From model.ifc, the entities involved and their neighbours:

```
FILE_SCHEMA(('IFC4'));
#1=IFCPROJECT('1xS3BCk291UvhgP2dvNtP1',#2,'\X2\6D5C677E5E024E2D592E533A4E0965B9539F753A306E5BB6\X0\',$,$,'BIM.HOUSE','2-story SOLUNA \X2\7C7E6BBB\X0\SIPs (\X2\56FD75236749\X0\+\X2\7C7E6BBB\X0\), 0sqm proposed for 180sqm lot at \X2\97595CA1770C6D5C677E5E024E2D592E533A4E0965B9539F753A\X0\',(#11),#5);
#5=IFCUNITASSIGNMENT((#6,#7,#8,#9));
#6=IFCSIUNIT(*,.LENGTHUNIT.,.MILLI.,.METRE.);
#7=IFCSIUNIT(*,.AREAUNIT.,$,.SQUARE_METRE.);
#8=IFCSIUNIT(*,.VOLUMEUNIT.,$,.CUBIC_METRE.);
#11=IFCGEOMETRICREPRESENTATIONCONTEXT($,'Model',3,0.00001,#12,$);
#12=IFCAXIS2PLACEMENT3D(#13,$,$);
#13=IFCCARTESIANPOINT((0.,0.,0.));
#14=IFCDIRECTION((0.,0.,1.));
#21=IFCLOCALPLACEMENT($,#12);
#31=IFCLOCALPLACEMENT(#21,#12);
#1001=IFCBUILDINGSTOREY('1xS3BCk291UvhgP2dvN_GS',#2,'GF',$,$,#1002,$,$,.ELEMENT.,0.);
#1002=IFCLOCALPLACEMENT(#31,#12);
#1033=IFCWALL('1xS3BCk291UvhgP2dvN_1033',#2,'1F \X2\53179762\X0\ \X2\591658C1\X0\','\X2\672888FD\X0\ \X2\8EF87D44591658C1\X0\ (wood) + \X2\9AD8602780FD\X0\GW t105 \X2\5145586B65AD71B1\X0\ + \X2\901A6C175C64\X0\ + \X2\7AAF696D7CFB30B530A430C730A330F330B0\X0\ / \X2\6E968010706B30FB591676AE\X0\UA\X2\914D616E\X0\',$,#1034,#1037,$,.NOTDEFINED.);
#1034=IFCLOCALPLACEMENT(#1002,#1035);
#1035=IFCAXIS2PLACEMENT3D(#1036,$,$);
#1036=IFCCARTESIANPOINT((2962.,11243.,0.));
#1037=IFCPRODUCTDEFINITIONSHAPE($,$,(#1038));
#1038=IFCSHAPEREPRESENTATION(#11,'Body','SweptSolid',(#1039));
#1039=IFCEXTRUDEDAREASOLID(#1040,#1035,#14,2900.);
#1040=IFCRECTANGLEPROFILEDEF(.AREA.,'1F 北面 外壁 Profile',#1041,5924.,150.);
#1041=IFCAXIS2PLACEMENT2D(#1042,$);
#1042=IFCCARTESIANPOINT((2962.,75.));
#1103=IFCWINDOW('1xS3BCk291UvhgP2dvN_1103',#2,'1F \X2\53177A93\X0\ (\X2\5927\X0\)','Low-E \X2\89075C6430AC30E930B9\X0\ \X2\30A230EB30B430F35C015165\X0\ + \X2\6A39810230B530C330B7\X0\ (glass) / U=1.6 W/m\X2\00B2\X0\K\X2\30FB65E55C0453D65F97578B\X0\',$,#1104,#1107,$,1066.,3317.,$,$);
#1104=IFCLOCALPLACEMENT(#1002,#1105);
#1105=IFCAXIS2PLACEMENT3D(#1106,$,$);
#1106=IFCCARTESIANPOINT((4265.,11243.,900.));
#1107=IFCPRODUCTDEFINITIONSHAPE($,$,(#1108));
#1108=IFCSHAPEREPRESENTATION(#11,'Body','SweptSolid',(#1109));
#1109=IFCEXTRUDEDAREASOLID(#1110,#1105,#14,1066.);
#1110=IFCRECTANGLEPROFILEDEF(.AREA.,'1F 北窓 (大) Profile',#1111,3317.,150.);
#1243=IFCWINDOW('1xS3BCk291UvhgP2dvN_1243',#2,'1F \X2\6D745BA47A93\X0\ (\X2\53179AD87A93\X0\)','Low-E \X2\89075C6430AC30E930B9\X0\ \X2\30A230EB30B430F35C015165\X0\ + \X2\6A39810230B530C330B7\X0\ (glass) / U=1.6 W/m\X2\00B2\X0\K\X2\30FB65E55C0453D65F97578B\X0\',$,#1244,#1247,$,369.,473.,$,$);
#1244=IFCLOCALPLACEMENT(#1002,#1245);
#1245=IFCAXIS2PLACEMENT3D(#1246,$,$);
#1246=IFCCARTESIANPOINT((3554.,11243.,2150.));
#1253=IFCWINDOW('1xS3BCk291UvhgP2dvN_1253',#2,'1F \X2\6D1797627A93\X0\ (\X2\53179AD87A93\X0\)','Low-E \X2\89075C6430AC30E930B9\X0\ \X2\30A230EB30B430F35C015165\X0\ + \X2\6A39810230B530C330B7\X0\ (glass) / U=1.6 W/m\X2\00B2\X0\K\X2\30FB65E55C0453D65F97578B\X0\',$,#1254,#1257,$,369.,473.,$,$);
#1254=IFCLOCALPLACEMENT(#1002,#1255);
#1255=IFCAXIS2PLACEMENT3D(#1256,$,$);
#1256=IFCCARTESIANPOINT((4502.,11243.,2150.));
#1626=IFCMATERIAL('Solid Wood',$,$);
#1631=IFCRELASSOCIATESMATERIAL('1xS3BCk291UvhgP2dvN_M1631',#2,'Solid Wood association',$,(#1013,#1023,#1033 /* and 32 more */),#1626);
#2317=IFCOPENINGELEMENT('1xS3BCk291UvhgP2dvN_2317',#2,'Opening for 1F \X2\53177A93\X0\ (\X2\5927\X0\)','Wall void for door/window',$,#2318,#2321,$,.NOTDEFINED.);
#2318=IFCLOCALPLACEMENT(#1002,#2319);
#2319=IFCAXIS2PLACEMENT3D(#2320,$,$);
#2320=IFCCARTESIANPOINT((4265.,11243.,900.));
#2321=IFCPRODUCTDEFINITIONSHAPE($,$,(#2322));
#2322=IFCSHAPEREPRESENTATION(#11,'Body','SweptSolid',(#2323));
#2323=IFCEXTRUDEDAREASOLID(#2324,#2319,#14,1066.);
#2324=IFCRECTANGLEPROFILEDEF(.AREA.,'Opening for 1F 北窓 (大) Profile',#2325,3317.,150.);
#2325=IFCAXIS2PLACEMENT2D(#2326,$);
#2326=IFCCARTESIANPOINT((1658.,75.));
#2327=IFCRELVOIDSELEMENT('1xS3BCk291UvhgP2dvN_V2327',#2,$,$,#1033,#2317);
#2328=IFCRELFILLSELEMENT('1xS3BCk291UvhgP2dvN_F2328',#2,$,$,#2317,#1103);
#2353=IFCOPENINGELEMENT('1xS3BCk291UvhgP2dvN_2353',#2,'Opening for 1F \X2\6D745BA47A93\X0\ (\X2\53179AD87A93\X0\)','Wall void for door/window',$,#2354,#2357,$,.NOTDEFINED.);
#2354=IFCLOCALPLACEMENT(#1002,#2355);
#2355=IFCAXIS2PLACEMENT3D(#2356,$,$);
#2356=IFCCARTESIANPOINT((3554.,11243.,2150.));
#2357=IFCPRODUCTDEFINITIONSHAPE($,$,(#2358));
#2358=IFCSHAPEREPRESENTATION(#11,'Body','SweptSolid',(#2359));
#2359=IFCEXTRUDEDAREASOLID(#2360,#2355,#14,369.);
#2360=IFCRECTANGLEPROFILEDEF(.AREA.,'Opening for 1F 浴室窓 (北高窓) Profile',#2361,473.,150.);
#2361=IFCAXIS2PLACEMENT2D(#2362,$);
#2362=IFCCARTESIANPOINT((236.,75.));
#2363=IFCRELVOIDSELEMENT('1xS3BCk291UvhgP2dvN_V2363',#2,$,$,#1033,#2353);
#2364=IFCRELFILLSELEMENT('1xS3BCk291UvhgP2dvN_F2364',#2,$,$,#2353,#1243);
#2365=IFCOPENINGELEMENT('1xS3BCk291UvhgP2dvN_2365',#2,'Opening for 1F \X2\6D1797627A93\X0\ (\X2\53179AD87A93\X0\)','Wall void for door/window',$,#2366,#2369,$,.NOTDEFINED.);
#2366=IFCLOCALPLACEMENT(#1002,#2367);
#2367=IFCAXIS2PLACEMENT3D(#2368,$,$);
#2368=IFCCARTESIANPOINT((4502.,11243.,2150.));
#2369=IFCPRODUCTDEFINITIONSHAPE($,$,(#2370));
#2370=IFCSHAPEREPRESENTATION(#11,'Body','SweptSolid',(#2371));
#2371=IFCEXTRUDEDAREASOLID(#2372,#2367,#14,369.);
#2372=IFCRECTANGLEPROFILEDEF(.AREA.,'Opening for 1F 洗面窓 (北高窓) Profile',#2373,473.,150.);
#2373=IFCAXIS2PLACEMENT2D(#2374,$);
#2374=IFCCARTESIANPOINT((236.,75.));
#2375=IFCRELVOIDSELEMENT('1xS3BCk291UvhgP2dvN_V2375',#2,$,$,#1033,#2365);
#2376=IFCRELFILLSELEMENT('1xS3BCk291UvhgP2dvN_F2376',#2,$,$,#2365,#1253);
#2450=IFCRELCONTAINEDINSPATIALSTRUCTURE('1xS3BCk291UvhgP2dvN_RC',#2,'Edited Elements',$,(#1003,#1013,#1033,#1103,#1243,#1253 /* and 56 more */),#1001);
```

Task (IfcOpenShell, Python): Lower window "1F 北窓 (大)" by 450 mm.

```python
import numpy as np
import ifcopenshell
import ifcopenshell.api.geometry
import ifcopenshell.util.placement
import ifcopenshell.util.unit

model = ifcopenshell.open("model.ifc")
unit_scale = ifcopenshell.util.unit.calculate_unit_scale(model)

window = model.by_guid("1xS3BCk291UvhgP2dvN_1103")
opening = window.FillsVoids[0].RelatingOpeningElement
dz = -450.0

shift = np.array([0.0, 0.0, dz])
# The window is not placed relative to its opening, so move both.
for product in (opening, window):
    matrix = ifcopenshell.util.placement.get_local_placement(product.ObjectPlacement)
    matrix[:3, 3] += shift
    ifcopenshell.api.geometry.edit_object_placement(model, product=product, matrix=matrix, is_si=False)

print(f"moved by {dz * unit_scale:+.3f} m")

model.write("model_edited.ifc")
```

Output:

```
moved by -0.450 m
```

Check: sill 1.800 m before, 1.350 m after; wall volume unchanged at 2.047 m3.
